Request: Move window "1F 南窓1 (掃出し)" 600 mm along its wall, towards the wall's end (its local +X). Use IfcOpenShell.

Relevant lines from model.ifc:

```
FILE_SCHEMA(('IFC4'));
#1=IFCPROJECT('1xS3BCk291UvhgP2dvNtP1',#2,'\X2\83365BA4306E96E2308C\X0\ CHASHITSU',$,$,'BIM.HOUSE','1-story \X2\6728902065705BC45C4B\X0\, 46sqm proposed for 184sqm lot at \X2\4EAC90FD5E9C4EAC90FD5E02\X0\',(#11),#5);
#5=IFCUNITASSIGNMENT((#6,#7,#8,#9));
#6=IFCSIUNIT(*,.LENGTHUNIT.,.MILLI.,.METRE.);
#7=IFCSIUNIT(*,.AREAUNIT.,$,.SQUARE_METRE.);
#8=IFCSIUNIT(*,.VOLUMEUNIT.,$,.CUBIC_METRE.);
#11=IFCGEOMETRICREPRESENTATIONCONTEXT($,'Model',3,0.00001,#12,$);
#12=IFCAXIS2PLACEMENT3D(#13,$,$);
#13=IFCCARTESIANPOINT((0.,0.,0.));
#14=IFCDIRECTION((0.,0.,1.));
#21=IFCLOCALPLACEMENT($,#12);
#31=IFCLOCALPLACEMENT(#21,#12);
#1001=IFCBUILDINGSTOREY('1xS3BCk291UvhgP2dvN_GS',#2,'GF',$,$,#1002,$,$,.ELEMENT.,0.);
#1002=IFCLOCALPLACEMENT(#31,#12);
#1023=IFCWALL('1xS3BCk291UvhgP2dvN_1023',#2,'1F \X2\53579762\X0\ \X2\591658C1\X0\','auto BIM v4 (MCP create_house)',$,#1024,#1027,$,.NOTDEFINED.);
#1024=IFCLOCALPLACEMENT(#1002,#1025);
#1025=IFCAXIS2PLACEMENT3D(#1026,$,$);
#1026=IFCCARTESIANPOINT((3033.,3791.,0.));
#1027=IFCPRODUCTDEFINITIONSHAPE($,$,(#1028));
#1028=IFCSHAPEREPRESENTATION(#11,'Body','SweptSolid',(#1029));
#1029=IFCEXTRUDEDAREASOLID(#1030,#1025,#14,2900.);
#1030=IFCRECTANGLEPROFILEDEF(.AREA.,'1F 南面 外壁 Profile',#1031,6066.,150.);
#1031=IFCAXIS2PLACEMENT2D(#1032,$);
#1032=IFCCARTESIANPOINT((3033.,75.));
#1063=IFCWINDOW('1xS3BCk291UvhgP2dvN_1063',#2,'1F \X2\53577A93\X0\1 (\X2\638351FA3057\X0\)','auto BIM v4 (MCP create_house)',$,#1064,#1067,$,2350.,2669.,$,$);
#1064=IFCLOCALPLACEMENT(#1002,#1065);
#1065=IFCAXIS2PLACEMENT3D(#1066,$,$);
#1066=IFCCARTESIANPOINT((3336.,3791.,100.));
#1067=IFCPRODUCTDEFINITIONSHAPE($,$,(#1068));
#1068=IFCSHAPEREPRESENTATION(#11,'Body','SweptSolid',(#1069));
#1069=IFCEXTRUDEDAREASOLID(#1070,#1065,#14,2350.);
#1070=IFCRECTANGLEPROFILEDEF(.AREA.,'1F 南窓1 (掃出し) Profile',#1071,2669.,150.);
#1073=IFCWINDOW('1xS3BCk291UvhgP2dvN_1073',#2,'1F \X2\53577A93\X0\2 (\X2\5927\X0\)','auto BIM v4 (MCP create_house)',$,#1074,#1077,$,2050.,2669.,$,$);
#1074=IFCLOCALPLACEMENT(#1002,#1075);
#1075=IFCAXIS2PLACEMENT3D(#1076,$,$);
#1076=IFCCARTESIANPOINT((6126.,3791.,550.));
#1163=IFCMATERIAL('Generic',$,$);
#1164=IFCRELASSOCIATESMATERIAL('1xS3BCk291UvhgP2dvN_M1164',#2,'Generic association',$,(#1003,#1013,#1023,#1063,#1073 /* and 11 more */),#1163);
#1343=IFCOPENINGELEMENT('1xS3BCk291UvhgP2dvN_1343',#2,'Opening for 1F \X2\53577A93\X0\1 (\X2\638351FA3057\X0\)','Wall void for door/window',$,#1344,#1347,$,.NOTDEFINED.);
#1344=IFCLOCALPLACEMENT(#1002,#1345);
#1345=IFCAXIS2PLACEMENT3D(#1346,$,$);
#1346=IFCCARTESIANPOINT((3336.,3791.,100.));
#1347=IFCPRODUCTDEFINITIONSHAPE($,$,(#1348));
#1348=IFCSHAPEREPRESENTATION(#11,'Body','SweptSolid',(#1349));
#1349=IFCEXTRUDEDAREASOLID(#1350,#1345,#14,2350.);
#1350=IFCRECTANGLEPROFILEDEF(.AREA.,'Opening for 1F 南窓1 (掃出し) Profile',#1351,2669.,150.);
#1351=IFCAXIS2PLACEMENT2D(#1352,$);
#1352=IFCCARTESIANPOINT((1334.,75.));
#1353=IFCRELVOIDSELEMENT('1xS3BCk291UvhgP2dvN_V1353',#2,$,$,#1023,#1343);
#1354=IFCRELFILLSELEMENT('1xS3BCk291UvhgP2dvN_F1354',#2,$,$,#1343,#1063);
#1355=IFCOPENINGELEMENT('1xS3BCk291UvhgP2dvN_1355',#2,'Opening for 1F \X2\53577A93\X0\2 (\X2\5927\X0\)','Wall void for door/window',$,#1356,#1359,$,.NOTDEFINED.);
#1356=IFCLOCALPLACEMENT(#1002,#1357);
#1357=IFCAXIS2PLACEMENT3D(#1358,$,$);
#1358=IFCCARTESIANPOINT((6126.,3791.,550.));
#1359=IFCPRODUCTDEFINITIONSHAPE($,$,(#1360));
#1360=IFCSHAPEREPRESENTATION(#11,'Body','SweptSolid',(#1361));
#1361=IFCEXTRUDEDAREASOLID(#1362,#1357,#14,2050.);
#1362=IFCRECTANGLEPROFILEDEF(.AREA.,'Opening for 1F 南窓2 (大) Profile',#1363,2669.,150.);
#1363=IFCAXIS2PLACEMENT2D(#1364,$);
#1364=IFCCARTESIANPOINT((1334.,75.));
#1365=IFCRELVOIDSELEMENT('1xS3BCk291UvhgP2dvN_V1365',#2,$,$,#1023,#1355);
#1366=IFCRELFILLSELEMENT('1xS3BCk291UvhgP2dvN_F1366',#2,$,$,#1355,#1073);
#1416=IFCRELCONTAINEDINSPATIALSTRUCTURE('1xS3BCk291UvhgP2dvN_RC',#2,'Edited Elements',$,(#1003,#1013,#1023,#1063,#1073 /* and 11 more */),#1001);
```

```python
import ifcopenshell
import ifcopenshell.api.geometry
import ifcopenshell.util.placement

model = ifcopenshell.open("model.ifc")

window = model.by_guid("1xS3BCk291UvhgP2dvN_1063")
opening = window.FillsVoids[0].RelatingOpeningElement
wall = opening.VoidsElements[0].RelatingBuildingElement

wall_matrix = ifcopenshell.util.placement.get_local_placement(wall.ObjectPlacement)
shift = wall_matrix[:3, 0] * 600.0
before = ifcopenshell.util.placement.get_local_placement(window.ObjectPlacement)[:3, 3].copy()

# The window is not placed relative to its opening, so move both.
for product in (opening, window):
    matrix = ifcopenshell.util.placement.get_local_placement(product.ObjectPlacement)
    matrix[:3, 3] += shift
    ifcopenshell.api.geometry.edit_object_placement(model, product=product, matrix=matrix, is_si=False)

after = ifcopenshell.util.placement.get_local_placement(window.ObjectPlacement)[:3, 3]
print("window moved by", (after - before).round(3) + 0.0)

model.write("model_rev.ifc")
```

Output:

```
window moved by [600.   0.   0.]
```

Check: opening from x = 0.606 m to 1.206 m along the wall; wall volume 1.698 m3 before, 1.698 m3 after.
